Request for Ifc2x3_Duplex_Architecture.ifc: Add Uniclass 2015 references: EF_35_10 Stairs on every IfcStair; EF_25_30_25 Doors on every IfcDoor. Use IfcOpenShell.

First a look at what the model holds.

```python
import ifcopenshell

model = ifcopenshell.open("Ifc2x3_Duplex_Architecture.ifc")
print(model.schema)
print("classifications:", [c.Name for c in model.by_type("IfcClassification")])
for ifc_class in ("IfcDoor", "IfcRoof", "IfcStair", "IfcWall", "IfcWindow"):
    print(ifc_class, len(model.by_type(ifc_class)))
```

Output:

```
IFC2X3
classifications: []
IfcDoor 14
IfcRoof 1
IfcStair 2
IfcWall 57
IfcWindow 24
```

```python
import ifcopenshell
import ifcopenshell.api.classification

model = ifcopenshell.open("Ifc2x3_Duplex_Architecture.ifc")

# IFC2X3 requires Source and Edition and has no link from the project to the system.
system = model.create_entity("IfcClassification", Source="NBS", Edition="2015", Name="Uniclass 2015")

codes = {
    "IfcStair": ("EF_35_10", "Stairs"),
    "IfcDoor": ("EF_25_30_25", "Doors"),
}
for ifc_class, (code, name) in codes.items():
    products = model.by_type(ifc_class)
    ifcopenshell.api.classification.add_reference(
        model, products=products, classification=system, identification=code, name=name
    )
    print(code, len(products))

model.write("Ifc2x3_Duplex_Architecture_rev.ifc")
```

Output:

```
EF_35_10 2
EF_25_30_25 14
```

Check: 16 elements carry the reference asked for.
